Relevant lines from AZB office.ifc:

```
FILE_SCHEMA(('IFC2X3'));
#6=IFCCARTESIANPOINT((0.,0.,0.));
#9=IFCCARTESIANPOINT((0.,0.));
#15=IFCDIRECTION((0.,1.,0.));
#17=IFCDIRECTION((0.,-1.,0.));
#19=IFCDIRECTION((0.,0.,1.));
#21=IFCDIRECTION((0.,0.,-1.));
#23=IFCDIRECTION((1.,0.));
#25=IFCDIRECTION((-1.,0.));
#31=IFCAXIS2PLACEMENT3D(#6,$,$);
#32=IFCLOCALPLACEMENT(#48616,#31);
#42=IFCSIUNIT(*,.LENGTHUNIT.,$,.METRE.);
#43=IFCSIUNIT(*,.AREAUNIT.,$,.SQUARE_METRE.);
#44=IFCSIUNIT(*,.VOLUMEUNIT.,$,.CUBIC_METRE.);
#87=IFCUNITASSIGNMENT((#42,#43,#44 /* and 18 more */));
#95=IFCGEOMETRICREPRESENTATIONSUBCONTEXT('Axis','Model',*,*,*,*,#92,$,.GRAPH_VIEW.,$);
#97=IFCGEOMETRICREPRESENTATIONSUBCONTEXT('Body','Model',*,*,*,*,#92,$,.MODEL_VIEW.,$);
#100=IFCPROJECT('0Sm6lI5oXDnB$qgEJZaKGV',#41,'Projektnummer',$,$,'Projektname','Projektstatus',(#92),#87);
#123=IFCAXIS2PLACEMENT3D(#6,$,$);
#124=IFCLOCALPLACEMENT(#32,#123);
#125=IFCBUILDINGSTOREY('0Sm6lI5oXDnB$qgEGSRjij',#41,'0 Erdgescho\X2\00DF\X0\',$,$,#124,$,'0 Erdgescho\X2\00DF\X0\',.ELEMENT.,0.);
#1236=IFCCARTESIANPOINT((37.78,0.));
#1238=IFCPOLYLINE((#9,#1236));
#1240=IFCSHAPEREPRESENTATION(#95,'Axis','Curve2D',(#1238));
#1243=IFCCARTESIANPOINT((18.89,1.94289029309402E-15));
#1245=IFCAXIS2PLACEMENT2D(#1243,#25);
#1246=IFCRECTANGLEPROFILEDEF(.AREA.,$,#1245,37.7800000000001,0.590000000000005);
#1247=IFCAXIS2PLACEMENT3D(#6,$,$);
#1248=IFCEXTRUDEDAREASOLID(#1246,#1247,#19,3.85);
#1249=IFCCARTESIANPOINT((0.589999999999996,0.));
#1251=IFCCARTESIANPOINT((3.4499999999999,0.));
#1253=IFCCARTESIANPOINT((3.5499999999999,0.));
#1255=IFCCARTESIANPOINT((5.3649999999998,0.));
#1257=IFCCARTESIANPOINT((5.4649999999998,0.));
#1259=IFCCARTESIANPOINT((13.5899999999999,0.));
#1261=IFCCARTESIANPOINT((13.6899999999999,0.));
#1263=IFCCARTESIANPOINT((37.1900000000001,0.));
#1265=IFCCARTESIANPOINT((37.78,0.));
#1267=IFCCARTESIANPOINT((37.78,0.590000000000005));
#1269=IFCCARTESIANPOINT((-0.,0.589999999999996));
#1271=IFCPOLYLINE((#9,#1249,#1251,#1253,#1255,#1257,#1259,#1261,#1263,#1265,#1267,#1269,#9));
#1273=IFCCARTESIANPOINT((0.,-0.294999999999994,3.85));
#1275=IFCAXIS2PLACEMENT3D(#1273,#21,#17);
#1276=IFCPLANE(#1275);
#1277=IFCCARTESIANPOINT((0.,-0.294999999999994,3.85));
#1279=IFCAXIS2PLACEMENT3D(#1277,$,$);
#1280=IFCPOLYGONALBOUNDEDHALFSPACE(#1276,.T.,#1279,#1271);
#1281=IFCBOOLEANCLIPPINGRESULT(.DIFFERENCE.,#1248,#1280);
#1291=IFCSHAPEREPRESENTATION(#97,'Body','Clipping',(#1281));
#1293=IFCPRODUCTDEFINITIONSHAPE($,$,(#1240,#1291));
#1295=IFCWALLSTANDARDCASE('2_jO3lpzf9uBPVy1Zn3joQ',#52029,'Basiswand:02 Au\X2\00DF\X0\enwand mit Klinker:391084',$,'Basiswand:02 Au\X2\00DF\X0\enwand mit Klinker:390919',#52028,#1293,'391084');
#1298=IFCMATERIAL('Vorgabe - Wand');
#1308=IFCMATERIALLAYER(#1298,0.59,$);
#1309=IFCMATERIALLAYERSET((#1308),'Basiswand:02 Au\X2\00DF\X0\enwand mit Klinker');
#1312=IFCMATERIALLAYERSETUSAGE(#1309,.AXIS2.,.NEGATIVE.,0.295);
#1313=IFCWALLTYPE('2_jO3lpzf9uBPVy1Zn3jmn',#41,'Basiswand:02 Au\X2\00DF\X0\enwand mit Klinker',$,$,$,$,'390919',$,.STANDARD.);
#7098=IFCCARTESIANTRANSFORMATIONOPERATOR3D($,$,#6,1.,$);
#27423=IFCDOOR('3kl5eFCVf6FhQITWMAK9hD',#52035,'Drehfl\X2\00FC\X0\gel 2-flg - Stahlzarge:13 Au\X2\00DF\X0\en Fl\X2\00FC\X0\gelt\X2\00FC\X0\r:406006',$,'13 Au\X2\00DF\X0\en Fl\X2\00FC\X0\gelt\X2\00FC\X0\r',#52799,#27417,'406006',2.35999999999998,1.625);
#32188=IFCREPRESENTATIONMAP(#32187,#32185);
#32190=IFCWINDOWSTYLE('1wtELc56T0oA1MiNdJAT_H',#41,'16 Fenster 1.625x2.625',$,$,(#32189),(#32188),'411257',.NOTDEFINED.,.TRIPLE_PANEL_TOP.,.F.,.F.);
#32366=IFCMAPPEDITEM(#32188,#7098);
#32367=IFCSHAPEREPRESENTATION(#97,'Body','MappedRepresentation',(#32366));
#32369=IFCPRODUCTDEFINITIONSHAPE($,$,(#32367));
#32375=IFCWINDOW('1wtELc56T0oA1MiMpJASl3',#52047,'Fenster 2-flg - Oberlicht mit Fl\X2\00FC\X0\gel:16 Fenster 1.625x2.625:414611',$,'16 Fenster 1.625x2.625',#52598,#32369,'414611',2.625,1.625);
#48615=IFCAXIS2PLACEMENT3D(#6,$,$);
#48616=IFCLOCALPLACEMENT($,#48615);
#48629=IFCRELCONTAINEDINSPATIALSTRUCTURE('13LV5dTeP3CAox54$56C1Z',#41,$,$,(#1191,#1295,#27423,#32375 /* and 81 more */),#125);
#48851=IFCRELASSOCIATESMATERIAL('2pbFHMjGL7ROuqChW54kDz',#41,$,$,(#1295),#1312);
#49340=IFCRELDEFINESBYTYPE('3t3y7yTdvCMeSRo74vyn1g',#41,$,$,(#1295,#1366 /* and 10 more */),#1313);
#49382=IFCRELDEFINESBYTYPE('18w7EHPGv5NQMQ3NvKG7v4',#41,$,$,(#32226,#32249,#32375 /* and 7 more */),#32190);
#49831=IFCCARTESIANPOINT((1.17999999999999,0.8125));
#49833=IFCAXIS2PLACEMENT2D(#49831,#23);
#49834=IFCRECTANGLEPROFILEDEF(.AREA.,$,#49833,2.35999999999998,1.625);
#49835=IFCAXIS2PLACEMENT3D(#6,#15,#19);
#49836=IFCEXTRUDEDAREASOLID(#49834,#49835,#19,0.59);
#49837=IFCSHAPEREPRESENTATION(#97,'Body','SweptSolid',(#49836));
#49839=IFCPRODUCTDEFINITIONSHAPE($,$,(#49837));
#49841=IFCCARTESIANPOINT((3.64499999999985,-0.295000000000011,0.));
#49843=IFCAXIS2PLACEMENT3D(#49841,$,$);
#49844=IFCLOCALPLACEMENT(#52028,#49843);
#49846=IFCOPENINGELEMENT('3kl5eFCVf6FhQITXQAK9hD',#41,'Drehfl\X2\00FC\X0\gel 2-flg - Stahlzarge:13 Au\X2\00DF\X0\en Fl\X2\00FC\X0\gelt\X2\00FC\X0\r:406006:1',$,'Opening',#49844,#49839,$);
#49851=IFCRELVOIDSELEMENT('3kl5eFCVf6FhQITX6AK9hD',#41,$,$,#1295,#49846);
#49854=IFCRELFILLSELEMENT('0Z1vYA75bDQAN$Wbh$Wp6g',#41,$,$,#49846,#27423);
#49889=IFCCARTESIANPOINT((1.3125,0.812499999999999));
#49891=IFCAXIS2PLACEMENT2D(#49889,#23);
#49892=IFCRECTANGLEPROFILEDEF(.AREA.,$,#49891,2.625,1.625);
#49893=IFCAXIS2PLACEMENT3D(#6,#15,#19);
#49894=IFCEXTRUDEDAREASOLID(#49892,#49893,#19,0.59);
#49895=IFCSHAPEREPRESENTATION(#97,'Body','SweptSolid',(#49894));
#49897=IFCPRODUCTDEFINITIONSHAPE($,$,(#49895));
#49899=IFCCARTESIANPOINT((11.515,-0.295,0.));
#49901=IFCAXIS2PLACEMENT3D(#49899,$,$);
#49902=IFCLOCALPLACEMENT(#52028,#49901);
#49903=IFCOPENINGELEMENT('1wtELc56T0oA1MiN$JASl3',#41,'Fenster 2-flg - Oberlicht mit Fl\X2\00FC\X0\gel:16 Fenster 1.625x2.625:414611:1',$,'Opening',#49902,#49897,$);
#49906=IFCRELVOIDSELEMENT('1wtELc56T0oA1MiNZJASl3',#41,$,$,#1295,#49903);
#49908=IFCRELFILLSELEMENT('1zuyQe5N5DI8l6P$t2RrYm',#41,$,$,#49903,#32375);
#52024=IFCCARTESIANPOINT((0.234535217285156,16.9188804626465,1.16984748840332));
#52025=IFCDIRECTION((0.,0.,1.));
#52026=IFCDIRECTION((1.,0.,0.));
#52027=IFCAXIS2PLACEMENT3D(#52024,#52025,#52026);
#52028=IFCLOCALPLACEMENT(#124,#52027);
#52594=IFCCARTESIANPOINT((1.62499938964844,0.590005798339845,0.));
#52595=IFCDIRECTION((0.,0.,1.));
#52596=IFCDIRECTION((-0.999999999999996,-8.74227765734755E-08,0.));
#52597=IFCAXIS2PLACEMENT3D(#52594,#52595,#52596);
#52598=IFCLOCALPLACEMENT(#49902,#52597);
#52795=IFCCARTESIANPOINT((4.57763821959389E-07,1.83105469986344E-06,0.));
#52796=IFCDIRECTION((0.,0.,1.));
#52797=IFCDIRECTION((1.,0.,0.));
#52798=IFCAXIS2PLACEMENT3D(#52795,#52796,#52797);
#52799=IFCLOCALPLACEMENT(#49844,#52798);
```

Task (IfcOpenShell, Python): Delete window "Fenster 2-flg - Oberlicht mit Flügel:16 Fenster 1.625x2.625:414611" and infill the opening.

```python
import ifcopenshell
import ifcopenshell.api.feature
import ifcopenshell.api.root
import ifcopenshell.geom
import ifcopenshell.util.shape

model = ifcopenshell.open("AZB office.ifc")
settings = ifcopenshell.geom.settings()


def volume(element):
    """Net volume in cubic metres, openings subtracted."""
    shape = ifcopenshell.geom.create_shape(settings, element)
    return ifcopenshell.util.shape.get_volume(shape.geometry)


window = model.by_guid("1wtELc56T0oA1MiMpJASl3")
opening = window.FillsVoids[0].RelatingOpeningElement
wall = opening.VoidsElements[0].RelatingBuildingElement
before = volume(wall)

ifcopenshell.api.root.remove_product(model, product=window)
ifcopenshell.api.feature.remove_feature(model, feature=opening)

after = volume(wall)

print(f"wall volume {before:.3f} -> {after:.3f} m3")

model.write("AZB office_edited.ifc")
```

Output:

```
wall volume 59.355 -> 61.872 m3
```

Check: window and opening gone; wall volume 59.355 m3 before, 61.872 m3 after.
